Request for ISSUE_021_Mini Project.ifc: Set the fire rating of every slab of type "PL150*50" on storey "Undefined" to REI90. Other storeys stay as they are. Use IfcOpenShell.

First a look at what the model holds.

```python
import ifcopenshell
import ifcopenshell.util.element

model = ifcopenshell.open("ISSUE_021_Mini Project.ifc")
print(model.schema)
storey = next(s for s in model.by_type("IfcBuildingStorey") if s.Name == "Undefined")
slabs = [e for e in ifcopenshell.util.element.get_decomposition(storey) if e.is_a("IfcSlab")]
seen = {}
for e in slabs:
    element_type = ifcopenshell.util.element.get_type(e)
    key = (element_type.Name if element_type != e and element_type else None, ifcopenshell.util.element.get_pset(e, "Pset_SlabCommon", "FireRating"))
    seen[key] = seen.get(key, 0) + 1
for (name, value), count in sorted(seen.items(), key=str):
    print(count, "x", name, "|", value)
```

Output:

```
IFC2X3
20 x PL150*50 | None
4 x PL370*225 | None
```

```python
import ifcopenshell
import ifcopenshell.api.pset
import ifcopenshell.util.element

model = ifcopenshell.open("ISSUE_021_Mini Project.ifc")

storey = next(s for s in model.by_type("IfcBuildingStorey") if s.Name == "Undefined")
slabs = [e for e in ifcopenshell.util.element.get_decomposition(storey) if e.is_a("IfcSlab")]

count = 0
for e in slabs:
    element_type = ifcopenshell.util.element.get_type(e)
    if element_type in (None, e) or element_type.Name != "PL150*50":
        continue
    found = ifcopenshell.util.element.get_pset(e, "Pset_SlabCommon", should_inherit=False)
    if found:
        pset = model.by_id(found["id"])
        if len(ifcopenshell.util.element.get_elements_by_pset(pset)) > 1:
            pset = ifcopenshell.api.pset.unshare_pset(model, products=[e], pset=pset)[0]
    else:
        pset = ifcopenshell.api.pset.add_pset(model, product=e, name="Pset_SlabCommon")
    ifcopenshell.api.pset.edit_pset(model, pset=pset, properties={"FireRating": "REI90"})
    count += 1

print(count, "slabs updated")

model.write("ISSUE_021_Mini Project-out.ifc")
```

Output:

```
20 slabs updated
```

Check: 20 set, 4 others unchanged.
